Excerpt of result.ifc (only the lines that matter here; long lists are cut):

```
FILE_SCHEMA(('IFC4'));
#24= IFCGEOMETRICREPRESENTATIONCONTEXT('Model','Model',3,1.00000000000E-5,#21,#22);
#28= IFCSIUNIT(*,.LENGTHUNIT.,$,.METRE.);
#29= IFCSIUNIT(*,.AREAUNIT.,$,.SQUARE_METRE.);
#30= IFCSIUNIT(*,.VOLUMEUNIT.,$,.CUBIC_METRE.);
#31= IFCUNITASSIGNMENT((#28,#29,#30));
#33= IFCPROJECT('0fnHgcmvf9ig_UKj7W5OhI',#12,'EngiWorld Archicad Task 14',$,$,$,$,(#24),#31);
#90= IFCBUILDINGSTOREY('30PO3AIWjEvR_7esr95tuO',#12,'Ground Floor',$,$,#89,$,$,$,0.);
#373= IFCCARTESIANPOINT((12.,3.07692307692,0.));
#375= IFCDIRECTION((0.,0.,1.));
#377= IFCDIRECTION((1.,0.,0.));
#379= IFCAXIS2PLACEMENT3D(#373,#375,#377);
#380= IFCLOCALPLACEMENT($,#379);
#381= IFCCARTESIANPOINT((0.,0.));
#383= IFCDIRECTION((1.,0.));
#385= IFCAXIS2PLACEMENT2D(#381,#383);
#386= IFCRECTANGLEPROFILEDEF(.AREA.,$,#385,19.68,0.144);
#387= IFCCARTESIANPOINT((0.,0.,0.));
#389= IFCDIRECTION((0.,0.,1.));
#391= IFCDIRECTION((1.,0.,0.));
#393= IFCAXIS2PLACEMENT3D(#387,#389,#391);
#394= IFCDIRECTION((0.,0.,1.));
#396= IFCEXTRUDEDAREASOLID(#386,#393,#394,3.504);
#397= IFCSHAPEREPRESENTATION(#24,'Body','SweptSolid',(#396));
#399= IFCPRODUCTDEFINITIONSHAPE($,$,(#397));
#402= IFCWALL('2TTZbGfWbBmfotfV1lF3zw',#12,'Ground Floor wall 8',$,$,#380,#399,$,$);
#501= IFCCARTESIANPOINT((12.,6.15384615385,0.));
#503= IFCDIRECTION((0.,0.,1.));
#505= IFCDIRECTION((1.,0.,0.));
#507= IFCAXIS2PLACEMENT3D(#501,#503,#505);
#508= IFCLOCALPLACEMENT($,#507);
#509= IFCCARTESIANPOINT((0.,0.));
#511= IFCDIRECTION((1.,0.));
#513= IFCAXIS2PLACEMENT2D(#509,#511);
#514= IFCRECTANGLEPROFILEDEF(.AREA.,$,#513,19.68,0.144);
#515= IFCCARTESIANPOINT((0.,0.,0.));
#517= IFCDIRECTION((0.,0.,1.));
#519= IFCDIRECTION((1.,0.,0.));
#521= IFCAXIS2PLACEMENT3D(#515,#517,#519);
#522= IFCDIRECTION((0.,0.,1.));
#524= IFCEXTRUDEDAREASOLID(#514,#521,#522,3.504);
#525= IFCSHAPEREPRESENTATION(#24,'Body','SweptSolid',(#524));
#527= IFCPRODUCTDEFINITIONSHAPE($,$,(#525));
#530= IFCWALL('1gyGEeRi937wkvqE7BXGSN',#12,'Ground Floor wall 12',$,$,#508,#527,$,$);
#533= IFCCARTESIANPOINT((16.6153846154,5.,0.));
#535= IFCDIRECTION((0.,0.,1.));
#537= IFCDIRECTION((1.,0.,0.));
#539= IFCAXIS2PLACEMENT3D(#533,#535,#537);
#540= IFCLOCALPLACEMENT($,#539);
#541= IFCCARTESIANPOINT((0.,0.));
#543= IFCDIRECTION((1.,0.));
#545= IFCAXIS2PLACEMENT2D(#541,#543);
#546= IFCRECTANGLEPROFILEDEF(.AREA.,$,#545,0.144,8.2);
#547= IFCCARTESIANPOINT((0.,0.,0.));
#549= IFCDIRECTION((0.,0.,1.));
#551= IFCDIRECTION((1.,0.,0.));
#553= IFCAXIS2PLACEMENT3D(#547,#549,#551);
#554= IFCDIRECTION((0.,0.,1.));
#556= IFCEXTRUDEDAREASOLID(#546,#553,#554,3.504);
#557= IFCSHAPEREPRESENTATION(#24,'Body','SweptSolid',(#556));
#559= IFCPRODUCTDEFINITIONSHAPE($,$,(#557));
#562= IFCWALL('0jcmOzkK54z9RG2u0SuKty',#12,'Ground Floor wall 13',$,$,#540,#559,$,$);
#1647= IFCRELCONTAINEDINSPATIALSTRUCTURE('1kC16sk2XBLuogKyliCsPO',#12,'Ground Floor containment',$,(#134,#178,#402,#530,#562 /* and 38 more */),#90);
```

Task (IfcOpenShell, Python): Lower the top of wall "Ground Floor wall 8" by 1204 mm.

```python
import ifcopenshell
import ifcopenshell.geom
import ifcopenshell.util.shape
import ifcopenshell.util.unit

model = ifcopenshell.open("result.ifc")
unit_scale = ifcopenshell.util.unit.calculate_unit_scale(model)
settings = ifcopenshell.geom.settings()


def volume(element):
    """Net volume in cubic metres, openings subtracted."""
    shape = ifcopenshell.geom.create_shape(settings, element)
    return ifcopenshell.util.shape.get_volume(shape.geometry)


wall = model.by_guid("2TTZbGfWbBmfotfV1lF3zw")
before = volume(wall)

body = next(r for r in wall.Representation.Representations if r.RepresentationIdentifier == "Body")
solid = body.Items[0]
old_height = solid.Depth
solid.Depth -= 1.204 / unit_scale
after = volume(wall)

print(f"height {old_height:g} -> {solid.Depth:g}, volume {before:.3f} -> {after:.3f} m3")

model.write("result_edited.ifc")
```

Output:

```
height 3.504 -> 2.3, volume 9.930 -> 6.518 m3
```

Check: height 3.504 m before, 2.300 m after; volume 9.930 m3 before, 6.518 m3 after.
